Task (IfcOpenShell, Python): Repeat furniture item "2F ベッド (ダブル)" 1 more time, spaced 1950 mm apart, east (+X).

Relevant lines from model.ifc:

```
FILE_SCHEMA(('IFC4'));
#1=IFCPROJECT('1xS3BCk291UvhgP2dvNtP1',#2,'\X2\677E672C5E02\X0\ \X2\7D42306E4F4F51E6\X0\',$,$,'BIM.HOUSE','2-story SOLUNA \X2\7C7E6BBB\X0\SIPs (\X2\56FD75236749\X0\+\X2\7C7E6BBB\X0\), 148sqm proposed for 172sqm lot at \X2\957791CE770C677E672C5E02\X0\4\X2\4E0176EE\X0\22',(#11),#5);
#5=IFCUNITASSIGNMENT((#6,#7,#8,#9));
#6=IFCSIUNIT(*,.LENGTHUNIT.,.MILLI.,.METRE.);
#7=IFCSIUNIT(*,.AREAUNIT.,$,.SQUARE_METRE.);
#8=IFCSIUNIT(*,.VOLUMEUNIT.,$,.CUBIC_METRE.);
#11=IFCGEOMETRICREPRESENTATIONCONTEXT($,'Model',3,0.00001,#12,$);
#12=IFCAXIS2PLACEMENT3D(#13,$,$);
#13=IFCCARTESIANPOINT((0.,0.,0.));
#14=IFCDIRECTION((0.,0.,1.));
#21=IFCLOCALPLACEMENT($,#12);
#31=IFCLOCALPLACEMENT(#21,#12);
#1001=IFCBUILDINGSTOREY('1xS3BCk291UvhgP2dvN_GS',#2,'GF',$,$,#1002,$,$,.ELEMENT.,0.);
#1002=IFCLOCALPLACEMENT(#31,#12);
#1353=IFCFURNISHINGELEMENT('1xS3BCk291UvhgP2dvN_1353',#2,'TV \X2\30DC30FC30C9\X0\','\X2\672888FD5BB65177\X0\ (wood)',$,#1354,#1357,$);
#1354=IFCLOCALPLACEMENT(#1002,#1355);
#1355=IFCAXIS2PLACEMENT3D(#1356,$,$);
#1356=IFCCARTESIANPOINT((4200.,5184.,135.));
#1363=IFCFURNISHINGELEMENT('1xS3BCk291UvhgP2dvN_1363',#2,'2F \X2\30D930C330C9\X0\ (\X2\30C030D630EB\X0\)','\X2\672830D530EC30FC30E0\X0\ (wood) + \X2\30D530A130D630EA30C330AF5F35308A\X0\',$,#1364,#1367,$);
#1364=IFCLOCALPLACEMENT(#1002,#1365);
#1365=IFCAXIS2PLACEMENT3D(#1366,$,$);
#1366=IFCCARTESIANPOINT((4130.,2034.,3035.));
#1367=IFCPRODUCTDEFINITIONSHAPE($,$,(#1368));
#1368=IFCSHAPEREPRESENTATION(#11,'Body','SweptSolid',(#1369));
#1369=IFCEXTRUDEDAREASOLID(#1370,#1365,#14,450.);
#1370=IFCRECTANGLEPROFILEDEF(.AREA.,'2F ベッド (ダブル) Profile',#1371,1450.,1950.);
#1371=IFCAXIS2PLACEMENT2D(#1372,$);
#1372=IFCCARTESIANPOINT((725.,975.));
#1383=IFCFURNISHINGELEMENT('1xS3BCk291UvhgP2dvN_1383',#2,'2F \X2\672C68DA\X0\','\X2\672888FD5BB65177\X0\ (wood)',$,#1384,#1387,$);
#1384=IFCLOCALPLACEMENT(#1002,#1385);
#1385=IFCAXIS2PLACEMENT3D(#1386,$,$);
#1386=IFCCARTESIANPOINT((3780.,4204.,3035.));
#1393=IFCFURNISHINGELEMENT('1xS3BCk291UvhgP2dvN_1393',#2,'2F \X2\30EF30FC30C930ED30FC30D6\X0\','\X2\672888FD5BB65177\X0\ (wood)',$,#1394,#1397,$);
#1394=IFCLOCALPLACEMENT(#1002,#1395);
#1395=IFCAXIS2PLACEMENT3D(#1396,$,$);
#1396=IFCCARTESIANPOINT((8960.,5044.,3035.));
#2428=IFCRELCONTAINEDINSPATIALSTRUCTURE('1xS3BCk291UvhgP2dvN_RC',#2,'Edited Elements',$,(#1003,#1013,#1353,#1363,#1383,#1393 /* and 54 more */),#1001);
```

```python
import numpy as np
import ifcopenshell
import ifcopenshell.api.geometry
import ifcopenshell.api.root
import ifcopenshell.util.element
import ifcopenshell.util.placement
import ifcopenshell.util.unit

model = ifcopenshell.open("model.ifc")
unit_scale = ifcopenshell.util.unit.calculate_unit_scale(model)


def reuse_history(source, copy):
    """copy_class also copies each property set's owner history, people and application; keep the originals."""
    for rel in copy.IsDefinedBy:
        if rel.is_a("IfcRelDefinesByProperties") and (history := rel.RelatingPropertyDefinition.OwnerHistory):
            rel.RelatingPropertyDefinition.OwnerHistory = source.OwnerHistory
            ifcopenshell.util.element.remove_deep2(model, history)


source = model.by_id(1363)
base = ifcopenshell.util.placement.get_local_placement(source.ObjectPlacement)
step = np.array([1.0, 0.0, 0.0]) * 1.95 / unit_scale

for i in range(1, 2):
    copy = ifcopenshell.api.root.copy_class(model, product=source)
    copy.Representation = ifcopenshell.util.element.copy_deep(
        model, source.Representation, exclude=["IfcGeometricRepresentationContext", "IfcRepresentationMap"]
    )
    reuse_history(source, copy)
    matrix = base.copy()
    matrix[:3, 3] += i * step
    print("added at", matrix[:3, 3].round(3) + 0.0)
    ifcopenshell.api.geometry.edit_object_placement(model, product=copy, matrix=matrix, is_si=False)

model.write("model-out.ifc")
```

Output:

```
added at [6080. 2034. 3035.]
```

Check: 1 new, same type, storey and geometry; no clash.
